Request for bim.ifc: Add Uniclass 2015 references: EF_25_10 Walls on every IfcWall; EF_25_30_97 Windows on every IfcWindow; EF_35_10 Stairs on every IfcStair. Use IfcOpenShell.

First a look at what the model holds.

```python
import ifcopenshell

model = ifcopenshell.open("bim.ifc")
print(model.schema)
print("classifications:", [c.Name for c in model.by_type("IfcClassification")])
for ifc_class in ("IfcDoor", "IfcRoof", "IfcStair", "IfcWall", "IfcWindow"):
    print(ifc_class, len(model.by_type(ifc_class)))
```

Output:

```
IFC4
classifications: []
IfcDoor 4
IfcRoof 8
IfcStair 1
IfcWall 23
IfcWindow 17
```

```python
import ifcopenshell
import ifcopenshell.api.classification

model = ifcopenshell.open("bim.ifc")

system = ifcopenshell.api.classification.add_classification(model, classification="Uniclass 2015")

codes = {
    "IfcWall": ("EF_25_10", "Walls"),
    "IfcWindow": ("EF_25_30_97", "Windows"),
    "IfcStair": ("EF_35_10", "Stairs"),
}
for ifc_class, (code, name) in codes.items():
    products = model.by_type(ifc_class)
    ifcopenshell.api.classification.add_reference(
        model, products=products, classification=system, identification=code, name=name
    )
    print(code, len(products))

model.write("bim_updated.ifc")
```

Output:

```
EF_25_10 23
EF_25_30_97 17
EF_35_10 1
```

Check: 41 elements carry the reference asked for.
